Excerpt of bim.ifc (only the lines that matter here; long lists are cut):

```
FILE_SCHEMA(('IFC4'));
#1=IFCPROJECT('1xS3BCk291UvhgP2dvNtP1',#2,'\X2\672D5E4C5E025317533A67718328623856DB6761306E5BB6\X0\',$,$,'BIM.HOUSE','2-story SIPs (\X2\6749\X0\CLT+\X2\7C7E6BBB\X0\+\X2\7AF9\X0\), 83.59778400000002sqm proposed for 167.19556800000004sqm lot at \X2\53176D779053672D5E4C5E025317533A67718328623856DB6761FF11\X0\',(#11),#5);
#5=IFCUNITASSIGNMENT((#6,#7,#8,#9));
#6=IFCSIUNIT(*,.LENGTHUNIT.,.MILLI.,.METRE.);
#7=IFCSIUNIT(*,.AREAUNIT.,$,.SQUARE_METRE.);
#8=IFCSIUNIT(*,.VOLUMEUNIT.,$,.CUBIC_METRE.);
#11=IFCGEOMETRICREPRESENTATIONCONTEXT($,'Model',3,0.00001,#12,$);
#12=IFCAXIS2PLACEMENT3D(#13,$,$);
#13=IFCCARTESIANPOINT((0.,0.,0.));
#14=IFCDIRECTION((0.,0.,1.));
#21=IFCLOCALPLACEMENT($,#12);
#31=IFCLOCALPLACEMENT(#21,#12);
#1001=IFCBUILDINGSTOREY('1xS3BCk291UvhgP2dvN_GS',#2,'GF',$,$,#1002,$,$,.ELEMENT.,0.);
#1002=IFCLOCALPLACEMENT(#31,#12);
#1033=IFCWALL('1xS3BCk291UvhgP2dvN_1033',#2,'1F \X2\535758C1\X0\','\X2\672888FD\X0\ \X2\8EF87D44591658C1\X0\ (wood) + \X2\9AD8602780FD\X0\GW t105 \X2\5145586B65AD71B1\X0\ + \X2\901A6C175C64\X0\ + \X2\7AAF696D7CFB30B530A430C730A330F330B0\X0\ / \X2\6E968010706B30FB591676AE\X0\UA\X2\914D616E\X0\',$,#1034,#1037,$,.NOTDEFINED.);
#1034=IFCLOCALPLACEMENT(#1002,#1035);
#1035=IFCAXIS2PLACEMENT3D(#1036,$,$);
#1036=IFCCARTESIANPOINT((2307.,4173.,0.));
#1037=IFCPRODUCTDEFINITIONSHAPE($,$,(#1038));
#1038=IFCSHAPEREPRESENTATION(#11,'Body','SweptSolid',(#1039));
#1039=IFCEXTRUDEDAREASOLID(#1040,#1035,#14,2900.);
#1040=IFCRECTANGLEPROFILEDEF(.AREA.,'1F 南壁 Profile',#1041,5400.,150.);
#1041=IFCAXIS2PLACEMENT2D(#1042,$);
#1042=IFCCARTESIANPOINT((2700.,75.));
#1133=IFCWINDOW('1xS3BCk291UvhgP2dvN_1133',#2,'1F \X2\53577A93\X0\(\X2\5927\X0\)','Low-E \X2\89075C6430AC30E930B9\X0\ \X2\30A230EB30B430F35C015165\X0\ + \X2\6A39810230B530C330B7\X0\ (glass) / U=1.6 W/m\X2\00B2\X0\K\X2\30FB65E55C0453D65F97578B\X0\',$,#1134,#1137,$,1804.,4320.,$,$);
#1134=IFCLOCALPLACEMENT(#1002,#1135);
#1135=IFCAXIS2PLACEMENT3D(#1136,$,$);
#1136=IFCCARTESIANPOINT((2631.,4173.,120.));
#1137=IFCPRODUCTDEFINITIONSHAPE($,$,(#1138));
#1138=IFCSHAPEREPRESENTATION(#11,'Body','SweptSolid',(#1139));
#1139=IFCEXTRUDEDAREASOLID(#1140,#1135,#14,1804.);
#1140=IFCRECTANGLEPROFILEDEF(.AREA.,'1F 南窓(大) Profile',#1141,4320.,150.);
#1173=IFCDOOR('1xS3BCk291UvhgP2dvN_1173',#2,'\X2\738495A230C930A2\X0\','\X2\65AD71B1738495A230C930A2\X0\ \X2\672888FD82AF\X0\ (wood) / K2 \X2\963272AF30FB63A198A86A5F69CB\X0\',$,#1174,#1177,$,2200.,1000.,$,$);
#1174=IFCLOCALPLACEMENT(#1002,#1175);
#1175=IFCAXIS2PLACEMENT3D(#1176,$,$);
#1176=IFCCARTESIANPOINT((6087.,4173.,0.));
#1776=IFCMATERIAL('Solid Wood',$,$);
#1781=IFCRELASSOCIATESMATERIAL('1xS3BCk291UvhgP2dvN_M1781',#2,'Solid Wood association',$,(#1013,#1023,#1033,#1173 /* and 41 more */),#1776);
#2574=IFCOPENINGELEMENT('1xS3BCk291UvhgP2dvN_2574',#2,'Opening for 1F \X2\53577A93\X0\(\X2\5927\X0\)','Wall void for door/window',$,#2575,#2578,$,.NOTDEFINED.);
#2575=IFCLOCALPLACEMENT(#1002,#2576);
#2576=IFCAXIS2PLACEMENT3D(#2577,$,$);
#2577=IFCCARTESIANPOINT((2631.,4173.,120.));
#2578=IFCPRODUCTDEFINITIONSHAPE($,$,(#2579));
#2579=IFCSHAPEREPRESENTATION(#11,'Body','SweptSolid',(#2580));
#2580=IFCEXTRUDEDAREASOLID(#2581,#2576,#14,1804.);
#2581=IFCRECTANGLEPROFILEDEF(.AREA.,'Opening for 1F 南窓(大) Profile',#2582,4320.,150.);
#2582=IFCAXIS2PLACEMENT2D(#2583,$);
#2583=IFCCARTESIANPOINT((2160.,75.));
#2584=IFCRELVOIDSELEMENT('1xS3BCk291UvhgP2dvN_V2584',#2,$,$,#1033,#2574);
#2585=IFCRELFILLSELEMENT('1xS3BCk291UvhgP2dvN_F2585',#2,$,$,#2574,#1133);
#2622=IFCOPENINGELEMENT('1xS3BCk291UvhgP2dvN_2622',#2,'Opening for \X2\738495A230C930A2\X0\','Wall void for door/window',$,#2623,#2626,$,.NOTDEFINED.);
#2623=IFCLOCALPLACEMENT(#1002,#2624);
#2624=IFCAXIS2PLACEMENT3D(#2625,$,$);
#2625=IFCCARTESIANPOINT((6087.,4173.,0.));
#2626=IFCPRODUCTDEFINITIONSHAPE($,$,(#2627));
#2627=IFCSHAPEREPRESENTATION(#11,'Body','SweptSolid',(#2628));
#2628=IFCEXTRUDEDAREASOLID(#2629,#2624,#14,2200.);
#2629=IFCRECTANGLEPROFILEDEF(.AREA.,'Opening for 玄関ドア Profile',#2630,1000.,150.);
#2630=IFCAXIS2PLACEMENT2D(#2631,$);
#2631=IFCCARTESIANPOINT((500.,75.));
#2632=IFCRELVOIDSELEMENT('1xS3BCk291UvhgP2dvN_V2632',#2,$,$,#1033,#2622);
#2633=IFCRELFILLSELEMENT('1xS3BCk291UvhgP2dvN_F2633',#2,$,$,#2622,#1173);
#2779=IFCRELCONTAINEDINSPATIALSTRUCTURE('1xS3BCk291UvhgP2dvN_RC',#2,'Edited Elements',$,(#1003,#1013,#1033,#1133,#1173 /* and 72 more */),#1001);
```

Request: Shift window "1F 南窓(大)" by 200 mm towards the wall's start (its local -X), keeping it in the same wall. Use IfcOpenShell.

```python
import ifcopenshell
import ifcopenshell.api.geometry
import ifcopenshell.util.placement
import ifcopenshell.util.unit

model = ifcopenshell.open("bim.ifc")
unit_scale = ifcopenshell.util.unit.calculate_unit_scale(model)

window = model.by_id(1133)
opening = window.FillsVoids[0].RelatingOpeningElement
wall = opening.VoidsElements[0].RelatingBuildingElement

wall_matrix = ifcopenshell.util.placement.get_local_placement(wall.ObjectPlacement)
shift = wall_matrix[:3, 0] * -0.2 / unit_scale
before = ifcopenshell.util.placement.get_local_placement(window.ObjectPlacement)[:3, 3].copy()

# The window is not placed relative to its opening, so move both.
for product in (opening, window):
    matrix = ifcopenshell.util.placement.get_local_placement(product.ObjectPlacement)
    matrix[:3, 3] += shift
    ifcopenshell.api.geometry.edit_object_placement(model, product=product, matrix=matrix, is_si=False)

after = ifcopenshell.util.placement.get_local_placement(window.ObjectPlacement)[:3, 3]
print("window moved by", (after - before).round(3) + 0.0)

model.write("bim_updated.ifc")
```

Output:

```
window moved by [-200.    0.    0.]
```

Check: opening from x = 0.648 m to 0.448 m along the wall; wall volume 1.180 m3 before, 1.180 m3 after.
